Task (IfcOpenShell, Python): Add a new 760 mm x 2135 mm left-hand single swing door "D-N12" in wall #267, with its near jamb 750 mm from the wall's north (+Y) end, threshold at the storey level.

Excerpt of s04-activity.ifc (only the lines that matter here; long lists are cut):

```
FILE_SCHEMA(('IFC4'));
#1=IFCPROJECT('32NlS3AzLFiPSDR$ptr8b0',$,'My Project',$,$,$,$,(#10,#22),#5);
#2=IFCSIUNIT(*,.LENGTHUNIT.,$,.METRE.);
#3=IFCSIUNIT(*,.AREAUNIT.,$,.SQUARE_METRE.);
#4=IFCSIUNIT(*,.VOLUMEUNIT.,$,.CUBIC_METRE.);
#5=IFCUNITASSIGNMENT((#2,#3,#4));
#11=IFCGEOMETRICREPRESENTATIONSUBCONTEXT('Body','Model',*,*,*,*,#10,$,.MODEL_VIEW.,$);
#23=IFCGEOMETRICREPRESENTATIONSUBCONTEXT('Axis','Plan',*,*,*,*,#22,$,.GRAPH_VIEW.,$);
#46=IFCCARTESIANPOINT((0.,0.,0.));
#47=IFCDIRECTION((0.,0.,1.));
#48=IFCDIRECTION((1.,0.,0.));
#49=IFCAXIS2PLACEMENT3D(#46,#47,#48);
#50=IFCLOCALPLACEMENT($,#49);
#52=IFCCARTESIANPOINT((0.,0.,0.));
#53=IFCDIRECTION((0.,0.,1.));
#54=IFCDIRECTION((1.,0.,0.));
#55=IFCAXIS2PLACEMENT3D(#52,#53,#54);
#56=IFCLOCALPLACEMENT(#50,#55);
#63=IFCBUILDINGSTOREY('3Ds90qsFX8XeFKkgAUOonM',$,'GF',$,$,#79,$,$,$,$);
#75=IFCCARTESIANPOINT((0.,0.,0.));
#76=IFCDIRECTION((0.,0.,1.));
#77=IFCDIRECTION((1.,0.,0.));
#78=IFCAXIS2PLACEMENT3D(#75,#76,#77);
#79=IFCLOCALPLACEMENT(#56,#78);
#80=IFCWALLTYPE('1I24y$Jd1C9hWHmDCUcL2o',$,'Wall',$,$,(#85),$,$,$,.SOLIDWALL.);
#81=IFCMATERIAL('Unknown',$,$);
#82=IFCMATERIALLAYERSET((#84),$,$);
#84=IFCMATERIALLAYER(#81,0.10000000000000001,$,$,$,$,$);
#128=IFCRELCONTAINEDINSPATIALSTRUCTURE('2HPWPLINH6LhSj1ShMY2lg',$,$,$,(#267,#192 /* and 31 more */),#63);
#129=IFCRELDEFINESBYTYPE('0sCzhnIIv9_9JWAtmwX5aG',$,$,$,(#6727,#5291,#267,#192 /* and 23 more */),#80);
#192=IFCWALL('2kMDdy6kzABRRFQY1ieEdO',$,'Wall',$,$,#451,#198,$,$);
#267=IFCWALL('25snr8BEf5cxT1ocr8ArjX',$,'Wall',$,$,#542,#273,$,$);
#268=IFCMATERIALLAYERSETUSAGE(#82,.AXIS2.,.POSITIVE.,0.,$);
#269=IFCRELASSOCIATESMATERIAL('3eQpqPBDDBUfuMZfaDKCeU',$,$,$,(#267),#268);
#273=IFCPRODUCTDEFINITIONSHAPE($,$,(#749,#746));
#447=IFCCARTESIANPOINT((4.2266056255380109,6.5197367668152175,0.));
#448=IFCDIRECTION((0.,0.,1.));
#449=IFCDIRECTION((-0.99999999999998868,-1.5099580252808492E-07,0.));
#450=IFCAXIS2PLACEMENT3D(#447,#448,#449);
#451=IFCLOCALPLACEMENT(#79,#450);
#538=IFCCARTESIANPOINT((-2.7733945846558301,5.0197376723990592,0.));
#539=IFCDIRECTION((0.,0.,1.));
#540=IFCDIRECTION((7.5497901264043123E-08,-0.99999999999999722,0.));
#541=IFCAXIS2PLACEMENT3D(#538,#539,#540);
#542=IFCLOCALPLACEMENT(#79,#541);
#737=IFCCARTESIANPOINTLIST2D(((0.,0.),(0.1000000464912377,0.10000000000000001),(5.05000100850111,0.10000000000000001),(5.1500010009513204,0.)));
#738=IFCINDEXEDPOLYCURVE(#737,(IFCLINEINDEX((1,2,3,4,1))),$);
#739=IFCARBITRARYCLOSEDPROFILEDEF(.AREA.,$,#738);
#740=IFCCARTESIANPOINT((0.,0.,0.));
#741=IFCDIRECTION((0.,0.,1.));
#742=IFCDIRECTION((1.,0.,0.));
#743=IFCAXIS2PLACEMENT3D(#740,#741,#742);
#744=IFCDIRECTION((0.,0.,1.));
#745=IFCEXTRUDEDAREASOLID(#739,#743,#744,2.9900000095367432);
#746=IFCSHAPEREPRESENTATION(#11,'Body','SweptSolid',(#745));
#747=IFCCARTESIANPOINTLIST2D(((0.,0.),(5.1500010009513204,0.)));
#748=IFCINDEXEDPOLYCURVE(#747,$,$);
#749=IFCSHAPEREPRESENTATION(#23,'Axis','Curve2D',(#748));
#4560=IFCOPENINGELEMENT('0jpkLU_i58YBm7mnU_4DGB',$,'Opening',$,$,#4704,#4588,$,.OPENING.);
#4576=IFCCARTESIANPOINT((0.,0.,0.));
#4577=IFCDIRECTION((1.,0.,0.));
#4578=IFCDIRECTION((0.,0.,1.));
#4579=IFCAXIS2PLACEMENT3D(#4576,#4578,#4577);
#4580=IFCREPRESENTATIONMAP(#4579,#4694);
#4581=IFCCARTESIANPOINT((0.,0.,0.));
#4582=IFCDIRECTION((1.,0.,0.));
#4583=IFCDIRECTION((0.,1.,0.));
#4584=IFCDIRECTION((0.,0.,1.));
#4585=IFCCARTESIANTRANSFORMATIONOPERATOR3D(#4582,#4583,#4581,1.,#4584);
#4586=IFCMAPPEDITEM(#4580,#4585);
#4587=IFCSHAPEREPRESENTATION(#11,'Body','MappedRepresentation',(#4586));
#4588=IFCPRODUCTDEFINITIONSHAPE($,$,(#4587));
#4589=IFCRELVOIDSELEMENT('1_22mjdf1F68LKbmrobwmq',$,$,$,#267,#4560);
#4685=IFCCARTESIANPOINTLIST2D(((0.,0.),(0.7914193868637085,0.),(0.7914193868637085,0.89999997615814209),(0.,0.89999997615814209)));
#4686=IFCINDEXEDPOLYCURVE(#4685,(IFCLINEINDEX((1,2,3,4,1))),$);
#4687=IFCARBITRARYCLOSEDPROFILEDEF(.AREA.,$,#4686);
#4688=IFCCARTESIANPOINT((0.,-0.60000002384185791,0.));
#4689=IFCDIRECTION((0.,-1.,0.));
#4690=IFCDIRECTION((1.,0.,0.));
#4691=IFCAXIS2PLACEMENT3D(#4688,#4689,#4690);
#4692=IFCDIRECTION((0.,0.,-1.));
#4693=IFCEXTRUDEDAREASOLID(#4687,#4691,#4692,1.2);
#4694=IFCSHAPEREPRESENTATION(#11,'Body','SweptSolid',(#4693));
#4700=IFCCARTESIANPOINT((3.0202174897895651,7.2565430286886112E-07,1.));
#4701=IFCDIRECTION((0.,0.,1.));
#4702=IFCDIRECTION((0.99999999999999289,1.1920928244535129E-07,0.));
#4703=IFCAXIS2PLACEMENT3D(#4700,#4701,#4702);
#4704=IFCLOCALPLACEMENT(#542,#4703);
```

```python
import numpy as np
import ifcopenshell
import ifcopenshell.api.feature
import ifcopenshell.api.geometry
import ifcopenshell.api.root
import ifcopenshell.api.spatial
import ifcopenshell.geom
import ifcopenshell.util.element
import ifcopenshell.util.placement
import ifcopenshell.util.representation
import ifcopenshell.util.shape
import ifcopenshell.util.unit

model = ifcopenshell.open("s04-activity.ifc")
unit_scale = ifcopenshell.util.unit.calculate_unit_scale(model)
settings = ifcopenshell.geom.settings()


def volume(element):
    """Net volume in cubic metres, openings subtracted."""
    shape = ifcopenshell.geom.create_shape(settings, element)
    return ifcopenshell.util.shape.get_volume(shape.geometry)


wall = model.by_guid("25snr8BEf5cxT1ocr8ArjX")
storey = ifcopenshell.util.element.get_container(wall, ifc_class="IfcBuildingStorey")
context = ifcopenshell.util.representation.get_context(model, "Model", "Body", "MODEL_VIEW")
before = volume(wall)

width, height, from_end, sill = 0.76, 2.135, 0.75, 0.0  # metres

# The wall runs along its own X axis, and the end named is its -X end.
wall_shape = ifcopenshell.geom.create_shape(settings, wall)
x, y, z = ifcopenshell.util.shape.get_vertices(wall_shape.geometry).T
start = x.min() + from_end
face, thickness = float(y.min()), float(y.max() - y.min())
wall_matrix = ifcopenshell.util.placement.get_local_placement(wall.ObjectPlacement)
level = ifcopenshell.util.placement.get_local_placement(storey.ObjectPlacement)[2, 3]


def in_wall(x, y):
    """Placement at x, y metres in the wall's axes, at sill height."""
    matrix = wall_matrix.copy()
    matrix[:, 3] = wall_matrix @ np.array([x / unit_scale, y / unit_scale, 0.0, 1.0])
    matrix[2, 3] = level + sill / unit_scale
    return matrix


# Opening: a box that overshoots both wall faces by 50 mm.
opening = ifcopenshell.api.root.create_entity(model, ifc_class="IfcOpeningElement", predefined_type="OPENING")
box = ifcopenshell.api.geometry.add_wall_representation(
    model, context=context, length=width, height=height, thickness=thickness + 0.1
)
ifcopenshell.api.geometry.assign_representation(model, product=opening, representation=box)
ifcopenshell.api.geometry.edit_object_placement(model, product=opening, matrix=in_wall(start, face - 0.05), is_si=False)
ifcopenshell.api.feature.add_feature(model, feature=opening, element=wall)

door = ifcopenshell.api.root.create_entity(model, ifc_class="IfcDoor", name="D-N12", predefined_type="DOOR")
door.OverallWidth, door.OverallHeight = width / unit_scale, height / unit_scale
door.OperationType = "SINGLE_SWING_LEFT"
body = ifcopenshell.api.geometry.add_door_representation(
    model,
    context=context,
    overall_width=door.OverallWidth,
    overall_height=door.OverallHeight,
    operation_type="SINGLE_SWING_LEFT",
    lining_properties={"LiningDepth": thickness / unit_scale, "ThresholdDepth": thickness / unit_scale},
)
ifcopenshell.api.geometry.assign_representation(model, product=door, representation=body)
ifcopenshell.api.spatial.assign_container(model, products=[door], relating_structure=storey)
ifcopenshell.api.feature.add_filling(model, opening=opening, element=door)

# The lining spans the wall, so the door starts at the wall face.
ifcopenshell.api.geometry.edit_object_placement(model, product=door, matrix=in_wall(start, face), is_si=False)

after = volume(wall)

print(f"wall volume {before:.3f} -> {after:.3f} m3")

model.write("s04-activity-out.ifc")
```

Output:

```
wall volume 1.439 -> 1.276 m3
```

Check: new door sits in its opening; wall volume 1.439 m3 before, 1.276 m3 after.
